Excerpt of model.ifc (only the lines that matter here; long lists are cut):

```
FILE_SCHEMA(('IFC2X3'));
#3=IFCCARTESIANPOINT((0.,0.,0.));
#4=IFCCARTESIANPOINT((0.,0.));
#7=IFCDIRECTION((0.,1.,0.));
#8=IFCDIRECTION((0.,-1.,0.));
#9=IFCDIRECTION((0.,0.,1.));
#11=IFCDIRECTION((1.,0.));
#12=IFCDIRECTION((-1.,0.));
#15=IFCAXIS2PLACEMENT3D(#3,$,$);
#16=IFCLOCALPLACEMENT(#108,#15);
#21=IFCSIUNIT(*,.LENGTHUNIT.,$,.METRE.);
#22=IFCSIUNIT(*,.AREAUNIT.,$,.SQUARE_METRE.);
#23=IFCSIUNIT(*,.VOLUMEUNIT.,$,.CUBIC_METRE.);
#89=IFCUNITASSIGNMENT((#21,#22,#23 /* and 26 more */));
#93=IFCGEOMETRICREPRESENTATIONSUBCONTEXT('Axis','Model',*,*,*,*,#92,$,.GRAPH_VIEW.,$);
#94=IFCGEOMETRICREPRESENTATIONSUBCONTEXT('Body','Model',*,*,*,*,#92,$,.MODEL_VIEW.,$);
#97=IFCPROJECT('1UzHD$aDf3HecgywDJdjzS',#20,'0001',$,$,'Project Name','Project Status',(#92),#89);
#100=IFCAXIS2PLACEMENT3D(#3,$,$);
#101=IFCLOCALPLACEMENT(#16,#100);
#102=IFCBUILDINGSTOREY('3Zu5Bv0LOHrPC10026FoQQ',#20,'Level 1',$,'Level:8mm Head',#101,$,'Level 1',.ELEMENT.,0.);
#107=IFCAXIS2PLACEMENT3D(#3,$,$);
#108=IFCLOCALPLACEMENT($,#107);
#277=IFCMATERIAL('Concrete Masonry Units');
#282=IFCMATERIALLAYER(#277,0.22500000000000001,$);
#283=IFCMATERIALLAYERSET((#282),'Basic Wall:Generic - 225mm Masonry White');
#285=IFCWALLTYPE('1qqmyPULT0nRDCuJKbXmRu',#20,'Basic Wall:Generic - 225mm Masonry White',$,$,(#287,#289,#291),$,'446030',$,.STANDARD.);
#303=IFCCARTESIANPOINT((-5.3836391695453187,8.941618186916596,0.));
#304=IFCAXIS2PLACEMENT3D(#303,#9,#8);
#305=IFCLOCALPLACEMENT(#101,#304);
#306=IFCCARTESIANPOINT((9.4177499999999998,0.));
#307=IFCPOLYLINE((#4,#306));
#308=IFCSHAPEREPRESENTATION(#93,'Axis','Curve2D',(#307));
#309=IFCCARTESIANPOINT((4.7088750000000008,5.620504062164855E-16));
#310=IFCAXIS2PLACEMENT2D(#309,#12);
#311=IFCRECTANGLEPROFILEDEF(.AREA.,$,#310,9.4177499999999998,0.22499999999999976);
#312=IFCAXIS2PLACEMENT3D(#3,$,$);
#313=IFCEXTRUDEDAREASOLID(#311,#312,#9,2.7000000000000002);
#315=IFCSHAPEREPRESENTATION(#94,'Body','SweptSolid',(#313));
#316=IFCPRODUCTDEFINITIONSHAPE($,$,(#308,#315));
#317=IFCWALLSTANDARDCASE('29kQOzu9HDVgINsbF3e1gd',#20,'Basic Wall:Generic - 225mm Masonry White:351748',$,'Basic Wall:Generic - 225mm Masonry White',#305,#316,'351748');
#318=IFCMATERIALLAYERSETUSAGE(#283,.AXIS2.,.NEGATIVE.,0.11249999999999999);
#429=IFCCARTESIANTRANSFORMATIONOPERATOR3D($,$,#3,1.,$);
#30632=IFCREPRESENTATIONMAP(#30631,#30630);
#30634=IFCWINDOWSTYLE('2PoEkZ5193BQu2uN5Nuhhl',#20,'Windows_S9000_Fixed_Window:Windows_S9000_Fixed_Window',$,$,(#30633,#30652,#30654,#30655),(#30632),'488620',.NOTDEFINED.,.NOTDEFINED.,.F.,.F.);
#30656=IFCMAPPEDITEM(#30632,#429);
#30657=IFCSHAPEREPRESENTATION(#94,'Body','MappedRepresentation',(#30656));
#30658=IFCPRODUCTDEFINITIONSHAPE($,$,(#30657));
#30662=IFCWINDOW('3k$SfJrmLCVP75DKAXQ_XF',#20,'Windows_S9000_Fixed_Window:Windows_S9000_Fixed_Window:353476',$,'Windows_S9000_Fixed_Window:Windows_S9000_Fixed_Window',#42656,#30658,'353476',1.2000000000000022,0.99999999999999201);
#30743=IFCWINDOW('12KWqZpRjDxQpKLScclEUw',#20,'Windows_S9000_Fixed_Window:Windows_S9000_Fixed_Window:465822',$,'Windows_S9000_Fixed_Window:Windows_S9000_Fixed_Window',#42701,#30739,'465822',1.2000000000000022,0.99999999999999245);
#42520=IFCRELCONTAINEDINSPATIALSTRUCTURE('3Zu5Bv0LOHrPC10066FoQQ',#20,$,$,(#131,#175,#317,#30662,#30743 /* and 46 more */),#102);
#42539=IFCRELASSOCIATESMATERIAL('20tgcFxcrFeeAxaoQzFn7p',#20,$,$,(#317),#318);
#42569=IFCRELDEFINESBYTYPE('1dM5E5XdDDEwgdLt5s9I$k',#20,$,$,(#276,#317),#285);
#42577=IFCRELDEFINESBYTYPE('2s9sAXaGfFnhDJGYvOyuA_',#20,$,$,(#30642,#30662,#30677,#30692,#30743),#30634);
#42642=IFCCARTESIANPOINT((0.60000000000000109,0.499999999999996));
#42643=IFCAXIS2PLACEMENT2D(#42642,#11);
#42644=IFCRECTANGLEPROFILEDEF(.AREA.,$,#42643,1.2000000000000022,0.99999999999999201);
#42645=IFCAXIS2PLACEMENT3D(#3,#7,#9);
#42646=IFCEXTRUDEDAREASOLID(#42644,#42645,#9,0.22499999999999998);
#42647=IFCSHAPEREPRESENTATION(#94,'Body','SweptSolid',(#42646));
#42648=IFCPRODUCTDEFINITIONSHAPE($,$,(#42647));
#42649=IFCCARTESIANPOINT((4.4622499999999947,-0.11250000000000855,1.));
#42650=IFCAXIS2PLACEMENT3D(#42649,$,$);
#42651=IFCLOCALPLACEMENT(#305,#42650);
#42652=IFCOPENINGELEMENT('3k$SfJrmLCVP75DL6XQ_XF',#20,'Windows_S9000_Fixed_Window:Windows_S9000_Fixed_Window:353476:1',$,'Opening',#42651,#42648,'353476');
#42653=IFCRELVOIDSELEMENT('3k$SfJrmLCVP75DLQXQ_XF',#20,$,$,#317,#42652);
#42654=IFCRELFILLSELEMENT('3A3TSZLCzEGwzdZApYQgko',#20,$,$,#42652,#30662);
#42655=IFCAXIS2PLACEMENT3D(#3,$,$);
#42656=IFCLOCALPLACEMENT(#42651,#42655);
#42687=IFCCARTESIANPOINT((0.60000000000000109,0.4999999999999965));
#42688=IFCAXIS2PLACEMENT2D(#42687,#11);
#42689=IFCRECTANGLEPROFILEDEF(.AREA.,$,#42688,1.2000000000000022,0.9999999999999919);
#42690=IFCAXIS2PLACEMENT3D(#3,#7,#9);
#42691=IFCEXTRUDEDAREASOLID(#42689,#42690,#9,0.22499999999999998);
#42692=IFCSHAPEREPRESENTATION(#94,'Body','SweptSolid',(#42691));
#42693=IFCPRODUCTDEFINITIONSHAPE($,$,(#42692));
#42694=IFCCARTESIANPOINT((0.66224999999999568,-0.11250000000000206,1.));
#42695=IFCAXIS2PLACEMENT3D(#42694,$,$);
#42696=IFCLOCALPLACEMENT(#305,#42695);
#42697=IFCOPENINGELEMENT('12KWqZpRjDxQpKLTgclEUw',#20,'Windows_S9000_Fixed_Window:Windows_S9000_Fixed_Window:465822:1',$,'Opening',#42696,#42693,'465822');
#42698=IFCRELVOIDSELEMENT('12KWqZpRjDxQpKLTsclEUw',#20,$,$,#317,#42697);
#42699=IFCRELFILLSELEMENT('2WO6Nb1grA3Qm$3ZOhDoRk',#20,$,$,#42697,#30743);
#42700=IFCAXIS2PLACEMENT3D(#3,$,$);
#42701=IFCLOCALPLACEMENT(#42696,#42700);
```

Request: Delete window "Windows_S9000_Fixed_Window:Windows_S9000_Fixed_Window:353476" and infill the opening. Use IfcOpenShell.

```python
import ifcopenshell
import ifcopenshell.api.feature
import ifcopenshell.api.root
import ifcopenshell.geom
import ifcopenshell.util.shape

model = ifcopenshell.open("model.ifc")
settings = ifcopenshell.geom.settings()


def volume(element):
    """Net volume in cubic metres, openings subtracted."""
    shape = ifcopenshell.geom.create_shape(settings, element)
    return ifcopenshell.util.shape.get_volume(shape.geometry)


window = model.by_id(30662)
opening = window.FillsVoids[0].RelatingOpeningElement
wall = opening.VoidsElements[0].RelatingBuildingElement
before = volume(wall)

ifcopenshell.api.root.remove_product(model, product=window)
ifcopenshell.api.feature.remove_feature(model, feature=opening)

after = volume(wall)

print(f"wall volume {before:.3f} -> {after:.3f} m3")

model.write("model_v2.ifc")
```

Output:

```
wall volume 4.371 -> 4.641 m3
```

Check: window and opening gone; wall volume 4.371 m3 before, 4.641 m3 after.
